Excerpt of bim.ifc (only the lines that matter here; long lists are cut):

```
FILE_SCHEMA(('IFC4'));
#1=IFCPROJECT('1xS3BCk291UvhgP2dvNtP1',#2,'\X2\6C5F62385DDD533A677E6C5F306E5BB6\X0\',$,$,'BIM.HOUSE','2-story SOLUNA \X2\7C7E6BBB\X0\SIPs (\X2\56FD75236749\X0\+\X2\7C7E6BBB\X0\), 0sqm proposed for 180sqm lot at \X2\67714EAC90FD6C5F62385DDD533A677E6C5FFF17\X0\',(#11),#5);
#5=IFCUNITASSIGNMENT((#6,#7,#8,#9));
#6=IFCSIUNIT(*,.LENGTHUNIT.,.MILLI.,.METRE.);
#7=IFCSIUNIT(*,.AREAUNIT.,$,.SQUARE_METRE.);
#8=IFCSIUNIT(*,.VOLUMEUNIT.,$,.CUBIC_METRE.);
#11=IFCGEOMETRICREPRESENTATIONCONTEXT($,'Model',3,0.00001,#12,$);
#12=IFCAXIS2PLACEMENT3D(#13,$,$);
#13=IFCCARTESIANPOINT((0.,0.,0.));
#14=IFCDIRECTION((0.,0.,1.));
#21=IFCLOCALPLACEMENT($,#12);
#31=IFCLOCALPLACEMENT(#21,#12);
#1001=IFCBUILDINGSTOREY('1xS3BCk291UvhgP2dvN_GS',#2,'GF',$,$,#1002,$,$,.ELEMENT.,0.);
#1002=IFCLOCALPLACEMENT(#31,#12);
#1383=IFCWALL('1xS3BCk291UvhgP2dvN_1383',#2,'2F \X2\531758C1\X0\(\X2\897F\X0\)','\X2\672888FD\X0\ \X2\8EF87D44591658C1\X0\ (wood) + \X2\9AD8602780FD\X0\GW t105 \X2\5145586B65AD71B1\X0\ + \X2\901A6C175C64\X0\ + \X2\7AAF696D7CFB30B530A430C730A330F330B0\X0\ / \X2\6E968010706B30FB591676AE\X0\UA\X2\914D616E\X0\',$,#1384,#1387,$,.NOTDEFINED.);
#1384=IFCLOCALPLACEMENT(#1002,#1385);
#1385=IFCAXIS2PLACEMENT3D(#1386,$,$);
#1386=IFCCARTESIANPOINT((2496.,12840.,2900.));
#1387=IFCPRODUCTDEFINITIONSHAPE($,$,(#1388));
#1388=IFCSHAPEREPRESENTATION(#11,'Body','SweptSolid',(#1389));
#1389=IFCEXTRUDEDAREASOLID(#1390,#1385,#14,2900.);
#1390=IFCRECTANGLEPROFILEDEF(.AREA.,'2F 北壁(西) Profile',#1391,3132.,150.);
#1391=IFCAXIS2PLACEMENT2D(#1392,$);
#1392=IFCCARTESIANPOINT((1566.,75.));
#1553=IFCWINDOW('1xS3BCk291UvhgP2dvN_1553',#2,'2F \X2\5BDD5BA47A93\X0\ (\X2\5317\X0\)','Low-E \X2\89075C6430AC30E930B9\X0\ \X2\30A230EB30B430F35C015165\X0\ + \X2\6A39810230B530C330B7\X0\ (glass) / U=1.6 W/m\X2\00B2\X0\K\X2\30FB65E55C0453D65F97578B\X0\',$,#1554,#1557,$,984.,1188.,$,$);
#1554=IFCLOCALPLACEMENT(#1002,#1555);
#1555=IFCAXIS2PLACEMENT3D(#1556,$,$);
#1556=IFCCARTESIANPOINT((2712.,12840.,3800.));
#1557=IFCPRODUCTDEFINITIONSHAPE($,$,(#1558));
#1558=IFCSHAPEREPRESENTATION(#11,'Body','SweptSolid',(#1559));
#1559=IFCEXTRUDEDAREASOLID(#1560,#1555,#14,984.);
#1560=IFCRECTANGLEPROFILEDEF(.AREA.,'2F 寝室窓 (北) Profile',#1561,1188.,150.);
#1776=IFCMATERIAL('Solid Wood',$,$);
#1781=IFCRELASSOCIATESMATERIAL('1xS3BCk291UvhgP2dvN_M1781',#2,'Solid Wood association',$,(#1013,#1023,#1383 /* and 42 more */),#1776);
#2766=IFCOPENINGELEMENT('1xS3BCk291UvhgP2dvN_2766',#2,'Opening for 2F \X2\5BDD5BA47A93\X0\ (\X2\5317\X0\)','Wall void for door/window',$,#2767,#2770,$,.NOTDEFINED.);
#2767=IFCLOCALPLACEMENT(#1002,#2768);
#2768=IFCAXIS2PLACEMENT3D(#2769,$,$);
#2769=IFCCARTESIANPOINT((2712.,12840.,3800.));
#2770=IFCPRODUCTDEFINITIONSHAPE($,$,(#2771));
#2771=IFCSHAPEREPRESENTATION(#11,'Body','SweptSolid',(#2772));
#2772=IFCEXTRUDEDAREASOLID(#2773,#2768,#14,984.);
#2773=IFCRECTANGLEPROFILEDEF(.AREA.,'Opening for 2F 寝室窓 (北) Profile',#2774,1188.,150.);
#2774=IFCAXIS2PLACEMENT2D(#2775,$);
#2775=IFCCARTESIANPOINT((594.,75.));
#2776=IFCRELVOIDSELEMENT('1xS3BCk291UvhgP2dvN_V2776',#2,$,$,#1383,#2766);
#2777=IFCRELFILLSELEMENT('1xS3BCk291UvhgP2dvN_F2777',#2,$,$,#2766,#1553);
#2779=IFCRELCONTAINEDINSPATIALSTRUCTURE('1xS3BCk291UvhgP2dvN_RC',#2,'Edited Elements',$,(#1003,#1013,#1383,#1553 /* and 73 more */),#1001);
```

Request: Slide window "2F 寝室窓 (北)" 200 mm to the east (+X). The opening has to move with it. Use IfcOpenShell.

```python
import ifcopenshell
import ifcopenshell.api.geometry
import ifcopenshell.util.placement
import ifcopenshell.util.unit

model = ifcopenshell.open("bim.ifc")
unit_scale = ifcopenshell.util.unit.calculate_unit_scale(model)

window = model.by_id(1553)
opening = window.FillsVoids[0].RelatingOpeningElement
wall = opening.VoidsElements[0].RelatingBuildingElement

wall_matrix = ifcopenshell.util.placement.get_local_placement(wall.ObjectPlacement)
shift = wall_matrix[:3, 0] * 0.2 / unit_scale
before = ifcopenshell.util.placement.get_local_placement(window.ObjectPlacement)[:3, 3].copy()

# The window is not placed relative to its opening, so move both.
for product in (opening, window):
    matrix = ifcopenshell.util.placement.get_local_placement(product.ObjectPlacement)
    matrix[:3, 3] += shift
    ifcopenshell.api.geometry.edit_object_placement(model, product=product, matrix=matrix, is_si=False)

after = ifcopenshell.util.placement.get_local_placement(window.ObjectPlacement)[:3, 3]
print("window moved by", (after - before).round(3) + 0.0)

model.write("bim_updated.ifc")
```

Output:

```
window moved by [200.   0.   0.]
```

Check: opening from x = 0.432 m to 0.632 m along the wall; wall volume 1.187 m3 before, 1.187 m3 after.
